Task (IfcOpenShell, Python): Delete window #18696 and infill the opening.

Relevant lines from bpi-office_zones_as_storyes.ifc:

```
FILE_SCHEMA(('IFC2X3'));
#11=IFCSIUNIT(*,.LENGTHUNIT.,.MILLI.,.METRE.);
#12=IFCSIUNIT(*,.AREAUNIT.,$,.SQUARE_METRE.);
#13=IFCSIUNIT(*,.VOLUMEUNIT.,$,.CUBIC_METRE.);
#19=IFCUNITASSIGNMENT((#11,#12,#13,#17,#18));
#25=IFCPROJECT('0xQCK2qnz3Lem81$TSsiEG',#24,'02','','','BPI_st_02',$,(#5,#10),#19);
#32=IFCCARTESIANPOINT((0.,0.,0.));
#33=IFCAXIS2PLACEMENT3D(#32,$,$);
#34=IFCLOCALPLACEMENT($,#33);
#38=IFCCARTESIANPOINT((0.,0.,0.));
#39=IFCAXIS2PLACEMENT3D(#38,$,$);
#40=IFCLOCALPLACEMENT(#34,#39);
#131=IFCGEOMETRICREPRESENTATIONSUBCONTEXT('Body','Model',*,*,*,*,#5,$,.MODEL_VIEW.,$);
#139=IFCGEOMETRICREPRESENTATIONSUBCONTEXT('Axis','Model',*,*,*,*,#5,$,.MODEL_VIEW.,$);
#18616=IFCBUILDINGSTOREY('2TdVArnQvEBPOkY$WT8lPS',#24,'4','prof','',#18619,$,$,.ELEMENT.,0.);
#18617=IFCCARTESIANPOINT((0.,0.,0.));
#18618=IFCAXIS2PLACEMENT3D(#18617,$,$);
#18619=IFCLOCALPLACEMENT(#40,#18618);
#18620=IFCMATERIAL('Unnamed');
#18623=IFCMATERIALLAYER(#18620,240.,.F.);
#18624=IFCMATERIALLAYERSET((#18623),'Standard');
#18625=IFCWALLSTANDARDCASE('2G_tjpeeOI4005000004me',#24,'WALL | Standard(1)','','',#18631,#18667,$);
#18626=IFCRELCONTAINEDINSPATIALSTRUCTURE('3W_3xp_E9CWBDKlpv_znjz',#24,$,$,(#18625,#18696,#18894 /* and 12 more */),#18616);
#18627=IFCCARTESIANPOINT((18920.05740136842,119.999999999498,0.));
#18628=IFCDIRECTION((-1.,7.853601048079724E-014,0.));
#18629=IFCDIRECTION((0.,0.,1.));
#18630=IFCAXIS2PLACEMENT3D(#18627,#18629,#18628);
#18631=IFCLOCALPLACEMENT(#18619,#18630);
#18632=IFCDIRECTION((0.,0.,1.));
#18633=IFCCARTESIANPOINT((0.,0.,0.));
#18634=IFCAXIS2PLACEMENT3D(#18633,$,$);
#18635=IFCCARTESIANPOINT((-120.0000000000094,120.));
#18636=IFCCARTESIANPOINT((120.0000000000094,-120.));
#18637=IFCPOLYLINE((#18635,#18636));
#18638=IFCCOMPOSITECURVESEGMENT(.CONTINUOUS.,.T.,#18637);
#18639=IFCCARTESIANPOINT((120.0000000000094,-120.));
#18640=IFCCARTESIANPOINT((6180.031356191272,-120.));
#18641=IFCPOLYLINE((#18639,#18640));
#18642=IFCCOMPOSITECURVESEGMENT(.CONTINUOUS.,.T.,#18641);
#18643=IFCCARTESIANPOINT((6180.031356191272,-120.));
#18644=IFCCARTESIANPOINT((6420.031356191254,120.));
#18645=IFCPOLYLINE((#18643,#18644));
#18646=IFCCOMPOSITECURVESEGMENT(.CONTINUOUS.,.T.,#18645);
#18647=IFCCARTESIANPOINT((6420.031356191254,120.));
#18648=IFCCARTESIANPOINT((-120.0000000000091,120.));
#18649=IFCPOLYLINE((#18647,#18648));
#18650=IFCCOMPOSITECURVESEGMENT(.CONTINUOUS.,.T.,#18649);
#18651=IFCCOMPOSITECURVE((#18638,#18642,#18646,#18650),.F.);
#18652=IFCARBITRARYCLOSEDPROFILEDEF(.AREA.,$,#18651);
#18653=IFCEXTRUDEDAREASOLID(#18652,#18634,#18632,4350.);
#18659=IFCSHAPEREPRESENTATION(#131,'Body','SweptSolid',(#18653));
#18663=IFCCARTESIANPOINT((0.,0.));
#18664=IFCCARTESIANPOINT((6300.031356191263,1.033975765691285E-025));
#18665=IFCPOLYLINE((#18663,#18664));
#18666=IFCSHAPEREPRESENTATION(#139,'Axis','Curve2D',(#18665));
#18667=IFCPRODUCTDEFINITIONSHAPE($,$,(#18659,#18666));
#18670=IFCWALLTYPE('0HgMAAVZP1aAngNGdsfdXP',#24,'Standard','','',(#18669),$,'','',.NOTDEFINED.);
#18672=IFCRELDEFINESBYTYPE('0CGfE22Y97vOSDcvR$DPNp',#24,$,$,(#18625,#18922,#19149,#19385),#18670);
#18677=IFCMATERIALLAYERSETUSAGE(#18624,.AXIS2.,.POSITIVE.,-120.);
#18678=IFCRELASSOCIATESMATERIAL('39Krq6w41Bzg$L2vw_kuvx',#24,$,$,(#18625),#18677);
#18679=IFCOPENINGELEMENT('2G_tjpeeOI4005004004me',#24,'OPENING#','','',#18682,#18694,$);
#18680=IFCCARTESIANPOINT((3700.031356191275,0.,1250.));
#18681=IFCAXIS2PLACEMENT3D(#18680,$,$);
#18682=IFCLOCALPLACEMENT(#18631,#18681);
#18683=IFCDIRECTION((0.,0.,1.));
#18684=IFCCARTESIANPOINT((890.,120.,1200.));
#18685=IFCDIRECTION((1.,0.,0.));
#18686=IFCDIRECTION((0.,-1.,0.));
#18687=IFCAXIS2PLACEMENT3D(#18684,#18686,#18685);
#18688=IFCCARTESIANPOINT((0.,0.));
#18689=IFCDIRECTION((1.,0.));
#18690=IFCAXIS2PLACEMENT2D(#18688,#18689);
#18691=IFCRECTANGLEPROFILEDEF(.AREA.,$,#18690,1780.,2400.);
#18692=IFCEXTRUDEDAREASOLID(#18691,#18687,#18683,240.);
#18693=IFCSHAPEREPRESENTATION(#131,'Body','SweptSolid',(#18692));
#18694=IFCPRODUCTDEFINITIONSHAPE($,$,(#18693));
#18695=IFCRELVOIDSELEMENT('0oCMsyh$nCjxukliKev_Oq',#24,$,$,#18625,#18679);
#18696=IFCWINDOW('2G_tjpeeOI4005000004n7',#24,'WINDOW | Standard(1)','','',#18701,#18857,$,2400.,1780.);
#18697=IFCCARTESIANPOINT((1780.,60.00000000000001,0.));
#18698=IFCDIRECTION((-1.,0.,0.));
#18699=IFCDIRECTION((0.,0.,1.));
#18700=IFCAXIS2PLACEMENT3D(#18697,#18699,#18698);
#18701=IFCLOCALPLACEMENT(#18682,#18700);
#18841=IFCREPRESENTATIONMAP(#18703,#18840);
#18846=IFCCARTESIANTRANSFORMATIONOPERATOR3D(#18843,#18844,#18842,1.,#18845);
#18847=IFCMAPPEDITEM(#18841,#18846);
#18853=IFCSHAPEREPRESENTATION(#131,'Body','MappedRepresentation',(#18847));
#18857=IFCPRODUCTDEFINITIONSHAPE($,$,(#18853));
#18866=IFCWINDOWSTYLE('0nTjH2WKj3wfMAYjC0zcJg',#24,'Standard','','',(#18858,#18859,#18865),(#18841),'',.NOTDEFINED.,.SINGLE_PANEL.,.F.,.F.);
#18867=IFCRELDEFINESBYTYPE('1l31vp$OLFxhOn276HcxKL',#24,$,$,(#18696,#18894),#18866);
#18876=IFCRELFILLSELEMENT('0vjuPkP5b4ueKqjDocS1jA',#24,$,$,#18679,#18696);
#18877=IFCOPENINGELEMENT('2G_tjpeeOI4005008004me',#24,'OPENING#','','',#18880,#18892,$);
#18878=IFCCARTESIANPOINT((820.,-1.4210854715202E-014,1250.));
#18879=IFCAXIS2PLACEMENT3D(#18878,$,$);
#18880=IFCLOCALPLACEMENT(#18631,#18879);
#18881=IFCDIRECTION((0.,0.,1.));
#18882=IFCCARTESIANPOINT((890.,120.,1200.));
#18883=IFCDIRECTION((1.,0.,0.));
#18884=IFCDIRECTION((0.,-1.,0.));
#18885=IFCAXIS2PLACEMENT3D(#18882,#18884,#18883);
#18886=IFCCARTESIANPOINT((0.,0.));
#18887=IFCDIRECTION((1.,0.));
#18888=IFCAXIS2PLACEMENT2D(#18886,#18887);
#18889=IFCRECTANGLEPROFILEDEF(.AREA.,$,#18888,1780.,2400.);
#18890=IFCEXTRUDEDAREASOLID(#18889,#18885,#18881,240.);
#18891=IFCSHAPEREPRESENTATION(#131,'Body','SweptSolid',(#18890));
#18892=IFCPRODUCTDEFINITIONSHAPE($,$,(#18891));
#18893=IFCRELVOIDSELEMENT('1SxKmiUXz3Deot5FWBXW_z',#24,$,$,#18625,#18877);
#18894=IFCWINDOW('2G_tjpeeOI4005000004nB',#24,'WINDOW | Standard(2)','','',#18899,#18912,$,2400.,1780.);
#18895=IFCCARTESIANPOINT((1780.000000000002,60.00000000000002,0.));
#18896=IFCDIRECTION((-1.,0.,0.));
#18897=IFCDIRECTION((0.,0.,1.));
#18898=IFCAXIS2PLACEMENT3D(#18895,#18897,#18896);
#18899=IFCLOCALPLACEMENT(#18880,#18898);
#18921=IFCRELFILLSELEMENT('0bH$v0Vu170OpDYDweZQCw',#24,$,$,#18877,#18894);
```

```python
import ifcopenshell
import ifcopenshell.api.feature
import ifcopenshell.api.root
import ifcopenshell.geom
import ifcopenshell.util.shape

model = ifcopenshell.open("bpi-office_zones_as_storyes.ifc")
settings = ifcopenshell.geom.settings()


def volume(element):
    """Net volume in cubic metres, openings subtracted."""
    shape = ifcopenshell.geom.create_shape(settings, element)
    return ifcopenshell.util.shape.get_volume(shape.geometry)


window = model.by_id(18696)
opening = window.FillsVoids[0].RelatingOpeningElement
wall = opening.VoidsElements[0].RelatingBuildingElement
before = volume(wall)

ifcopenshell.api.root.remove_product(model, product=window)
ifcopenshell.api.feature.remove_feature(model, feature=opening)

after = volume(wall)

print(f"wall volume {before:.3f} -> {after:.3f} m3")

model.write("bpi-office_zones_as_storyes_updated.ifc")
```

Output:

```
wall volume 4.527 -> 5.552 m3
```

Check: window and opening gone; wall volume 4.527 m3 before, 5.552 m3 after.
